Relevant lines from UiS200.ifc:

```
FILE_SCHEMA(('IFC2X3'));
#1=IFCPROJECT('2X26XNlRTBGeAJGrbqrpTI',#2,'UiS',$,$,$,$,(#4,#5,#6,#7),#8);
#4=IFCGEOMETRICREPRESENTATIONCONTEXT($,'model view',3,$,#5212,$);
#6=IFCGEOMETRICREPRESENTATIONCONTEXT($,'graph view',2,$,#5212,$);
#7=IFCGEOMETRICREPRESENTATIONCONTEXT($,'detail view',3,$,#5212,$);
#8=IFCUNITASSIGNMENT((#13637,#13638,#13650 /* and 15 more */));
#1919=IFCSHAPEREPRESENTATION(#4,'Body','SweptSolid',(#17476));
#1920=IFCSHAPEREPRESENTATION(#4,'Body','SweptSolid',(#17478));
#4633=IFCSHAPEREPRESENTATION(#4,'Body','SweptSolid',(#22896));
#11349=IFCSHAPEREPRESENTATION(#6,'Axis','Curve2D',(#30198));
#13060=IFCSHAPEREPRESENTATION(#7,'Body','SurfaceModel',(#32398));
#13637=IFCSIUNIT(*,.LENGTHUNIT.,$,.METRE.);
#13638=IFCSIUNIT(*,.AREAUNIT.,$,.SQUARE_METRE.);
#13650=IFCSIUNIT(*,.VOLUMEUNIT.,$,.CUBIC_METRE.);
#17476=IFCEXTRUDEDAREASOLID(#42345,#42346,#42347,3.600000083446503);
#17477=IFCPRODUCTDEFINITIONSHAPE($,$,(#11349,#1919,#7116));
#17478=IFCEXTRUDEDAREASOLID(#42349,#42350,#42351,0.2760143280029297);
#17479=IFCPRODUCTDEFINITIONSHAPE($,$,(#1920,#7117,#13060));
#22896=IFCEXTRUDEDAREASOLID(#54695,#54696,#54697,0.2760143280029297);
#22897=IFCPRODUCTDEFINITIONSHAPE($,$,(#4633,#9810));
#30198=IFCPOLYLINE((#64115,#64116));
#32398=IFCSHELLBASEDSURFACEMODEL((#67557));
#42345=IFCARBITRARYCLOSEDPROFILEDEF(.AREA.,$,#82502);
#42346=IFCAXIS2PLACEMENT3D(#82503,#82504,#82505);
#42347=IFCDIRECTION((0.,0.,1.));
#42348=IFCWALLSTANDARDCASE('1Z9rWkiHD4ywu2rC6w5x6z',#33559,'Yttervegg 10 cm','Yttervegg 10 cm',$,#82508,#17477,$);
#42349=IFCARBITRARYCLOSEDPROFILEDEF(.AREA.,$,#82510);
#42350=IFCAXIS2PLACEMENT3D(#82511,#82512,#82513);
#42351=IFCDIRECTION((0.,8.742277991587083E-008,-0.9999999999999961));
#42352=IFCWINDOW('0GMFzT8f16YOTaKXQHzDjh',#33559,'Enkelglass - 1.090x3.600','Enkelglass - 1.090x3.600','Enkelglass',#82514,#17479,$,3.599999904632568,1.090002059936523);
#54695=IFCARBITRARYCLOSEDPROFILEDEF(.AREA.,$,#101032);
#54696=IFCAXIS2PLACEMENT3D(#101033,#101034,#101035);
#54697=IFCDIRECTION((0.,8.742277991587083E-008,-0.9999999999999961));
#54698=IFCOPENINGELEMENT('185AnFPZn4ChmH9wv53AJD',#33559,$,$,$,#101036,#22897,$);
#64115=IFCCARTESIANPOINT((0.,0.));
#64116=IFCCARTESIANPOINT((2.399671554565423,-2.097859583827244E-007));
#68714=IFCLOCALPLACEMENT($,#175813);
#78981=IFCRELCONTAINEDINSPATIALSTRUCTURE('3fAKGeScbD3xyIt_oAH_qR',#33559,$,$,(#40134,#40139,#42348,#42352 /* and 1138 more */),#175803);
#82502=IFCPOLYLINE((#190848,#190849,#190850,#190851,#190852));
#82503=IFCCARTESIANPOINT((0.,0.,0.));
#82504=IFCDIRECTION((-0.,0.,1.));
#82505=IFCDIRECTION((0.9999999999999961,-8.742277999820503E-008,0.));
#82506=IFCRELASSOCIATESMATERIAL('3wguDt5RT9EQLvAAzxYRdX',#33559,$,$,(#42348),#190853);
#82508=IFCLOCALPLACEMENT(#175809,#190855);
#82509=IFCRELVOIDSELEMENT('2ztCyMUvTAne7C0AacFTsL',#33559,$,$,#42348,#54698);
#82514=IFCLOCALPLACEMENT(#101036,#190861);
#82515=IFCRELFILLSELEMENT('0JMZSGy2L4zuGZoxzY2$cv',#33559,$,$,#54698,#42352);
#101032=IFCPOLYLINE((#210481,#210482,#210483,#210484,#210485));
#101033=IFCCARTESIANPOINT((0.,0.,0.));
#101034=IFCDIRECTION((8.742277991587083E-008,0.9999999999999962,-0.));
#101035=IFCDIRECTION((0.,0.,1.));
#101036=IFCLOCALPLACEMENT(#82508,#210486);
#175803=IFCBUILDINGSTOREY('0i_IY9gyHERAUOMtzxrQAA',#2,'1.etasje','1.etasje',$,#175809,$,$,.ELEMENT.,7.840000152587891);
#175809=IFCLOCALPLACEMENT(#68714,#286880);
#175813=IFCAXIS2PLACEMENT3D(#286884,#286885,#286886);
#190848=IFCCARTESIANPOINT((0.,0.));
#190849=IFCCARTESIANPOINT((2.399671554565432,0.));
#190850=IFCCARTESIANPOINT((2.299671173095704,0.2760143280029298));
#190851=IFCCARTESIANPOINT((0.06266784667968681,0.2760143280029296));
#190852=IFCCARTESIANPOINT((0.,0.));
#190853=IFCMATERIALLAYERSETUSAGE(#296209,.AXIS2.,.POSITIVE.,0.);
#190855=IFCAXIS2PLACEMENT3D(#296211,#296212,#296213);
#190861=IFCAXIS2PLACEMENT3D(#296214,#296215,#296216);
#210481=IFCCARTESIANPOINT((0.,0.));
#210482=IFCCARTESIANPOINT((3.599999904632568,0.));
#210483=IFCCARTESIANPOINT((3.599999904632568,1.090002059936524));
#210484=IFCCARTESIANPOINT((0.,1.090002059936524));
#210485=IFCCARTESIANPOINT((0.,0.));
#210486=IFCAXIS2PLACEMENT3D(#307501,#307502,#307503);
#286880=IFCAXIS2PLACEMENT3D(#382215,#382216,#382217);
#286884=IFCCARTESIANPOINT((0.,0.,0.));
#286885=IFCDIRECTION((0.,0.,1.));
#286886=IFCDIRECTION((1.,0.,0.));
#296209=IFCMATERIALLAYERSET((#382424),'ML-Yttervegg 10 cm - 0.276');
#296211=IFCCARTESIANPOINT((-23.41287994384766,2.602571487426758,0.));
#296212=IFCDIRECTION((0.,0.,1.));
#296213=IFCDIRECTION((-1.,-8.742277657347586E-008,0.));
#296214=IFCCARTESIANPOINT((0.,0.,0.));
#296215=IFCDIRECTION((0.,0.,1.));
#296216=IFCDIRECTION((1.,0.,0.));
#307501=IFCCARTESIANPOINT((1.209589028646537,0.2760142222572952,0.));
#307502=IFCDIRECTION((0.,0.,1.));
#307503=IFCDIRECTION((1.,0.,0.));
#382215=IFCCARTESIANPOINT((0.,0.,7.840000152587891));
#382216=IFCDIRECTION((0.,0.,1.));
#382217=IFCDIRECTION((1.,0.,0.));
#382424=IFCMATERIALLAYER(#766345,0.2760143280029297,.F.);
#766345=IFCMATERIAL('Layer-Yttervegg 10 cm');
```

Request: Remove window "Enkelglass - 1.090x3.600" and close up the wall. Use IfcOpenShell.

```python
import ifcopenshell
import ifcopenshell.api.feature
import ifcopenshell.api.root
import ifcopenshell.geom
import ifcopenshell.util.shape

model = ifcopenshell.open("UiS200.ifc")
settings = ifcopenshell.geom.settings()


def volume(element):
    """Net volume in cubic metres, openings subtracted."""
    shape = ifcopenshell.geom.create_shape(settings, element)
    return ifcopenshell.util.shape.get_volume(shape.geometry)


window = model.by_id(42352)
opening = window.FillsVoids[0].RelatingOpeningElement
wall = opening.VoidsElements[0].RelatingBuildingElement
before = volume(wall)

ifcopenshell.api.root.remove_product(model, product=window)
ifcopenshell.api.feature.remove_feature(model, feature=opening)

after = volume(wall)

print(f"wall volume {before:.3f} -> {after:.3f} m3")

model.write("UiS200_updated.ifc")
```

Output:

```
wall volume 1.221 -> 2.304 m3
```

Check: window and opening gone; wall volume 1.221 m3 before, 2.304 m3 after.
